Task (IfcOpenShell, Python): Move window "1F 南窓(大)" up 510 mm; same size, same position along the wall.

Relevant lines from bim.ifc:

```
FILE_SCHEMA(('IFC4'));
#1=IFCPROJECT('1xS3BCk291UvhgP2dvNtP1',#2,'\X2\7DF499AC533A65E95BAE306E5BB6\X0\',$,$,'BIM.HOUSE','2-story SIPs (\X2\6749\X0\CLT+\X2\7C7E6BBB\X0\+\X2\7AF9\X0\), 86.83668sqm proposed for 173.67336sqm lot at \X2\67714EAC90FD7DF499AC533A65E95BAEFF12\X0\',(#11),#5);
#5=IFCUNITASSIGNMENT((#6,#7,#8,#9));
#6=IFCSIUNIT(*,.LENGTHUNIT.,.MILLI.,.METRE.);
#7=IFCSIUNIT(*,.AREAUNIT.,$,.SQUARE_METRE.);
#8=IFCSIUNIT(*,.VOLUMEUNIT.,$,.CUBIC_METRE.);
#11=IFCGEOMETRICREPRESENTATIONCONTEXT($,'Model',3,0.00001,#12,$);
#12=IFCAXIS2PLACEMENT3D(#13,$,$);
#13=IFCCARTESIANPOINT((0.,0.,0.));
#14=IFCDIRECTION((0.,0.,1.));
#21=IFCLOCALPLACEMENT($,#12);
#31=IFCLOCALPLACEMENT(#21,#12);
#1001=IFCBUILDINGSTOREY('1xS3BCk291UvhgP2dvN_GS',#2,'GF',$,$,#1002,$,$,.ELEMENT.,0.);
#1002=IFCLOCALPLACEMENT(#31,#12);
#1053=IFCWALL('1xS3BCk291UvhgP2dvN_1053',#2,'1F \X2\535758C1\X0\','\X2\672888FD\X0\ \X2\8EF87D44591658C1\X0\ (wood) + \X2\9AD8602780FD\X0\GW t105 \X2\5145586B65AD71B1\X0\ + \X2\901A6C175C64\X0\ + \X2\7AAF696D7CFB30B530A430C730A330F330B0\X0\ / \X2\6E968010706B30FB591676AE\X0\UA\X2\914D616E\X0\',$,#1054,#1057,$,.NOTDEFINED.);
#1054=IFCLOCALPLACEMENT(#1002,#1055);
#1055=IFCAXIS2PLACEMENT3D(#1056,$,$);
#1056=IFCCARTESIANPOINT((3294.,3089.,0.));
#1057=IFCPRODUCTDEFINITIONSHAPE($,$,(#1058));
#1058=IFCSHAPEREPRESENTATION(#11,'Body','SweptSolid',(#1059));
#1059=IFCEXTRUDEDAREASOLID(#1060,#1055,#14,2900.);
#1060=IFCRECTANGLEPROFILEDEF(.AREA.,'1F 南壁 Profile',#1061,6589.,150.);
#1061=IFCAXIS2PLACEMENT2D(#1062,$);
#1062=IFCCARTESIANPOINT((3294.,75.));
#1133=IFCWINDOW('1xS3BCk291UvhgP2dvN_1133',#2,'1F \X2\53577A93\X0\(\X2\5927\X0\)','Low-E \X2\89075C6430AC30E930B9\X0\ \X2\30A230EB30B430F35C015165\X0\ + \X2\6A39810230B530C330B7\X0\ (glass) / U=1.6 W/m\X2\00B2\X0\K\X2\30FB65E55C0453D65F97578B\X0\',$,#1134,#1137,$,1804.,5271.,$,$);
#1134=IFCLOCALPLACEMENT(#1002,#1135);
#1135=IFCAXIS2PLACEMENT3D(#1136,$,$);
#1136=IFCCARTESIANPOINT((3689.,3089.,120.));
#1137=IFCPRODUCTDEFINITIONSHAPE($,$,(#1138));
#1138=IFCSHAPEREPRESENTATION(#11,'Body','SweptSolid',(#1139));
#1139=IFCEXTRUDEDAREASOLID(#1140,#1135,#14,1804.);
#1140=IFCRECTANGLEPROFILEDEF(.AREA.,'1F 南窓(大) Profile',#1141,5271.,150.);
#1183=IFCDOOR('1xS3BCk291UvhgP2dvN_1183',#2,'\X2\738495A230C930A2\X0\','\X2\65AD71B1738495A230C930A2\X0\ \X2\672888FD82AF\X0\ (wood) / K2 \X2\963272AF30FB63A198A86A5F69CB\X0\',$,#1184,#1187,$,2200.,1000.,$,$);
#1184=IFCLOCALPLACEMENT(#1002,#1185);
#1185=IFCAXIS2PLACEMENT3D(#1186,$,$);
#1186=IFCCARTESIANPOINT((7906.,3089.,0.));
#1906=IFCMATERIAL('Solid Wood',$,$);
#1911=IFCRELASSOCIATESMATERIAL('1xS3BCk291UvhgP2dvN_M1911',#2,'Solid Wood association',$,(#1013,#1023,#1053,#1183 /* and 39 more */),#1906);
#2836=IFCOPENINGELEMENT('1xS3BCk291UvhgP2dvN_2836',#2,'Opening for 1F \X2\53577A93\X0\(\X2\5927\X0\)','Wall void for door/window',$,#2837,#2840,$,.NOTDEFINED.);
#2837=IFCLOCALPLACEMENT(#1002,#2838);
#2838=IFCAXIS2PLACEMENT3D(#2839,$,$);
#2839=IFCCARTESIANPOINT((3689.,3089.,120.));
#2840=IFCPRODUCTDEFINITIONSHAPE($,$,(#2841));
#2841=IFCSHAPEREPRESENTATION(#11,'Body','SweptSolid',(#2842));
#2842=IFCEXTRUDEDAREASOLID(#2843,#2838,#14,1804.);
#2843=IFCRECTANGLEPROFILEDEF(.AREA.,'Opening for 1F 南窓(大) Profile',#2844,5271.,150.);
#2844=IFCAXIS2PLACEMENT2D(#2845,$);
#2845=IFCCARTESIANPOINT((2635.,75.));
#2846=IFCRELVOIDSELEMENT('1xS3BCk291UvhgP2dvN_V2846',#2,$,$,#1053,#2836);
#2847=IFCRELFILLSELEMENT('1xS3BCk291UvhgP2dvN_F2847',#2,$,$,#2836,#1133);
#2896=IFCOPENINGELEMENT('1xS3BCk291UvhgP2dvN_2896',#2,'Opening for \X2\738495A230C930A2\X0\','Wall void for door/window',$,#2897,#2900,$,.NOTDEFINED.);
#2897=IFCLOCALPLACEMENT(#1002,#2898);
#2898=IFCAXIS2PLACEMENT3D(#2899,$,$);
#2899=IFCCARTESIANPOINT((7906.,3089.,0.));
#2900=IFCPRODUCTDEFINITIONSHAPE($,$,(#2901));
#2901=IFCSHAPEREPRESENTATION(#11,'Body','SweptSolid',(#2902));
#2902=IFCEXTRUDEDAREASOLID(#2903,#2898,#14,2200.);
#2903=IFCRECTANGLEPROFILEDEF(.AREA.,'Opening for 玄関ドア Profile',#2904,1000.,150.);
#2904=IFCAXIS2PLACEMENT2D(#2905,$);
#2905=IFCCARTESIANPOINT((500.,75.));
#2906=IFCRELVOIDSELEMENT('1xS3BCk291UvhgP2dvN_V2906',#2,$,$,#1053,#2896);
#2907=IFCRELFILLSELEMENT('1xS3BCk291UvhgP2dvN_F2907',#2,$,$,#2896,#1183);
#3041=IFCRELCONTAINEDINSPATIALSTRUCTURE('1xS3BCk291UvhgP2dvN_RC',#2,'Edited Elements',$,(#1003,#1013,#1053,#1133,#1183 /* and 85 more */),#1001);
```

```python
import numpy as np
import ifcopenshell
import ifcopenshell.api.geometry
import ifcopenshell.util.placement
import ifcopenshell.util.unit

model = ifcopenshell.open("bim.ifc")
unit_scale = ifcopenshell.util.unit.calculate_unit_scale(model)

window = model.by_id(1133)
opening = window.FillsVoids[0].RelatingOpeningElement
dz = 510.0

shift = np.array([0.0, 0.0, dz])
# The window is not placed relative to its opening, so move both.
for product in (opening, window):
    matrix = ifcopenshell.util.placement.get_local_placement(product.ObjectPlacement)
    matrix[:3, 3] += shift
    ifcopenshell.api.geometry.edit_object_placement(model, product=product, matrix=matrix, is_si=False)

print(f"moved by {dz * unit_scale:+.3f} m")

model.write("bim_v2.ifc")
```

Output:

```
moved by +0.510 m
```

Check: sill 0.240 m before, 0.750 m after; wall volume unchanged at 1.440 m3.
